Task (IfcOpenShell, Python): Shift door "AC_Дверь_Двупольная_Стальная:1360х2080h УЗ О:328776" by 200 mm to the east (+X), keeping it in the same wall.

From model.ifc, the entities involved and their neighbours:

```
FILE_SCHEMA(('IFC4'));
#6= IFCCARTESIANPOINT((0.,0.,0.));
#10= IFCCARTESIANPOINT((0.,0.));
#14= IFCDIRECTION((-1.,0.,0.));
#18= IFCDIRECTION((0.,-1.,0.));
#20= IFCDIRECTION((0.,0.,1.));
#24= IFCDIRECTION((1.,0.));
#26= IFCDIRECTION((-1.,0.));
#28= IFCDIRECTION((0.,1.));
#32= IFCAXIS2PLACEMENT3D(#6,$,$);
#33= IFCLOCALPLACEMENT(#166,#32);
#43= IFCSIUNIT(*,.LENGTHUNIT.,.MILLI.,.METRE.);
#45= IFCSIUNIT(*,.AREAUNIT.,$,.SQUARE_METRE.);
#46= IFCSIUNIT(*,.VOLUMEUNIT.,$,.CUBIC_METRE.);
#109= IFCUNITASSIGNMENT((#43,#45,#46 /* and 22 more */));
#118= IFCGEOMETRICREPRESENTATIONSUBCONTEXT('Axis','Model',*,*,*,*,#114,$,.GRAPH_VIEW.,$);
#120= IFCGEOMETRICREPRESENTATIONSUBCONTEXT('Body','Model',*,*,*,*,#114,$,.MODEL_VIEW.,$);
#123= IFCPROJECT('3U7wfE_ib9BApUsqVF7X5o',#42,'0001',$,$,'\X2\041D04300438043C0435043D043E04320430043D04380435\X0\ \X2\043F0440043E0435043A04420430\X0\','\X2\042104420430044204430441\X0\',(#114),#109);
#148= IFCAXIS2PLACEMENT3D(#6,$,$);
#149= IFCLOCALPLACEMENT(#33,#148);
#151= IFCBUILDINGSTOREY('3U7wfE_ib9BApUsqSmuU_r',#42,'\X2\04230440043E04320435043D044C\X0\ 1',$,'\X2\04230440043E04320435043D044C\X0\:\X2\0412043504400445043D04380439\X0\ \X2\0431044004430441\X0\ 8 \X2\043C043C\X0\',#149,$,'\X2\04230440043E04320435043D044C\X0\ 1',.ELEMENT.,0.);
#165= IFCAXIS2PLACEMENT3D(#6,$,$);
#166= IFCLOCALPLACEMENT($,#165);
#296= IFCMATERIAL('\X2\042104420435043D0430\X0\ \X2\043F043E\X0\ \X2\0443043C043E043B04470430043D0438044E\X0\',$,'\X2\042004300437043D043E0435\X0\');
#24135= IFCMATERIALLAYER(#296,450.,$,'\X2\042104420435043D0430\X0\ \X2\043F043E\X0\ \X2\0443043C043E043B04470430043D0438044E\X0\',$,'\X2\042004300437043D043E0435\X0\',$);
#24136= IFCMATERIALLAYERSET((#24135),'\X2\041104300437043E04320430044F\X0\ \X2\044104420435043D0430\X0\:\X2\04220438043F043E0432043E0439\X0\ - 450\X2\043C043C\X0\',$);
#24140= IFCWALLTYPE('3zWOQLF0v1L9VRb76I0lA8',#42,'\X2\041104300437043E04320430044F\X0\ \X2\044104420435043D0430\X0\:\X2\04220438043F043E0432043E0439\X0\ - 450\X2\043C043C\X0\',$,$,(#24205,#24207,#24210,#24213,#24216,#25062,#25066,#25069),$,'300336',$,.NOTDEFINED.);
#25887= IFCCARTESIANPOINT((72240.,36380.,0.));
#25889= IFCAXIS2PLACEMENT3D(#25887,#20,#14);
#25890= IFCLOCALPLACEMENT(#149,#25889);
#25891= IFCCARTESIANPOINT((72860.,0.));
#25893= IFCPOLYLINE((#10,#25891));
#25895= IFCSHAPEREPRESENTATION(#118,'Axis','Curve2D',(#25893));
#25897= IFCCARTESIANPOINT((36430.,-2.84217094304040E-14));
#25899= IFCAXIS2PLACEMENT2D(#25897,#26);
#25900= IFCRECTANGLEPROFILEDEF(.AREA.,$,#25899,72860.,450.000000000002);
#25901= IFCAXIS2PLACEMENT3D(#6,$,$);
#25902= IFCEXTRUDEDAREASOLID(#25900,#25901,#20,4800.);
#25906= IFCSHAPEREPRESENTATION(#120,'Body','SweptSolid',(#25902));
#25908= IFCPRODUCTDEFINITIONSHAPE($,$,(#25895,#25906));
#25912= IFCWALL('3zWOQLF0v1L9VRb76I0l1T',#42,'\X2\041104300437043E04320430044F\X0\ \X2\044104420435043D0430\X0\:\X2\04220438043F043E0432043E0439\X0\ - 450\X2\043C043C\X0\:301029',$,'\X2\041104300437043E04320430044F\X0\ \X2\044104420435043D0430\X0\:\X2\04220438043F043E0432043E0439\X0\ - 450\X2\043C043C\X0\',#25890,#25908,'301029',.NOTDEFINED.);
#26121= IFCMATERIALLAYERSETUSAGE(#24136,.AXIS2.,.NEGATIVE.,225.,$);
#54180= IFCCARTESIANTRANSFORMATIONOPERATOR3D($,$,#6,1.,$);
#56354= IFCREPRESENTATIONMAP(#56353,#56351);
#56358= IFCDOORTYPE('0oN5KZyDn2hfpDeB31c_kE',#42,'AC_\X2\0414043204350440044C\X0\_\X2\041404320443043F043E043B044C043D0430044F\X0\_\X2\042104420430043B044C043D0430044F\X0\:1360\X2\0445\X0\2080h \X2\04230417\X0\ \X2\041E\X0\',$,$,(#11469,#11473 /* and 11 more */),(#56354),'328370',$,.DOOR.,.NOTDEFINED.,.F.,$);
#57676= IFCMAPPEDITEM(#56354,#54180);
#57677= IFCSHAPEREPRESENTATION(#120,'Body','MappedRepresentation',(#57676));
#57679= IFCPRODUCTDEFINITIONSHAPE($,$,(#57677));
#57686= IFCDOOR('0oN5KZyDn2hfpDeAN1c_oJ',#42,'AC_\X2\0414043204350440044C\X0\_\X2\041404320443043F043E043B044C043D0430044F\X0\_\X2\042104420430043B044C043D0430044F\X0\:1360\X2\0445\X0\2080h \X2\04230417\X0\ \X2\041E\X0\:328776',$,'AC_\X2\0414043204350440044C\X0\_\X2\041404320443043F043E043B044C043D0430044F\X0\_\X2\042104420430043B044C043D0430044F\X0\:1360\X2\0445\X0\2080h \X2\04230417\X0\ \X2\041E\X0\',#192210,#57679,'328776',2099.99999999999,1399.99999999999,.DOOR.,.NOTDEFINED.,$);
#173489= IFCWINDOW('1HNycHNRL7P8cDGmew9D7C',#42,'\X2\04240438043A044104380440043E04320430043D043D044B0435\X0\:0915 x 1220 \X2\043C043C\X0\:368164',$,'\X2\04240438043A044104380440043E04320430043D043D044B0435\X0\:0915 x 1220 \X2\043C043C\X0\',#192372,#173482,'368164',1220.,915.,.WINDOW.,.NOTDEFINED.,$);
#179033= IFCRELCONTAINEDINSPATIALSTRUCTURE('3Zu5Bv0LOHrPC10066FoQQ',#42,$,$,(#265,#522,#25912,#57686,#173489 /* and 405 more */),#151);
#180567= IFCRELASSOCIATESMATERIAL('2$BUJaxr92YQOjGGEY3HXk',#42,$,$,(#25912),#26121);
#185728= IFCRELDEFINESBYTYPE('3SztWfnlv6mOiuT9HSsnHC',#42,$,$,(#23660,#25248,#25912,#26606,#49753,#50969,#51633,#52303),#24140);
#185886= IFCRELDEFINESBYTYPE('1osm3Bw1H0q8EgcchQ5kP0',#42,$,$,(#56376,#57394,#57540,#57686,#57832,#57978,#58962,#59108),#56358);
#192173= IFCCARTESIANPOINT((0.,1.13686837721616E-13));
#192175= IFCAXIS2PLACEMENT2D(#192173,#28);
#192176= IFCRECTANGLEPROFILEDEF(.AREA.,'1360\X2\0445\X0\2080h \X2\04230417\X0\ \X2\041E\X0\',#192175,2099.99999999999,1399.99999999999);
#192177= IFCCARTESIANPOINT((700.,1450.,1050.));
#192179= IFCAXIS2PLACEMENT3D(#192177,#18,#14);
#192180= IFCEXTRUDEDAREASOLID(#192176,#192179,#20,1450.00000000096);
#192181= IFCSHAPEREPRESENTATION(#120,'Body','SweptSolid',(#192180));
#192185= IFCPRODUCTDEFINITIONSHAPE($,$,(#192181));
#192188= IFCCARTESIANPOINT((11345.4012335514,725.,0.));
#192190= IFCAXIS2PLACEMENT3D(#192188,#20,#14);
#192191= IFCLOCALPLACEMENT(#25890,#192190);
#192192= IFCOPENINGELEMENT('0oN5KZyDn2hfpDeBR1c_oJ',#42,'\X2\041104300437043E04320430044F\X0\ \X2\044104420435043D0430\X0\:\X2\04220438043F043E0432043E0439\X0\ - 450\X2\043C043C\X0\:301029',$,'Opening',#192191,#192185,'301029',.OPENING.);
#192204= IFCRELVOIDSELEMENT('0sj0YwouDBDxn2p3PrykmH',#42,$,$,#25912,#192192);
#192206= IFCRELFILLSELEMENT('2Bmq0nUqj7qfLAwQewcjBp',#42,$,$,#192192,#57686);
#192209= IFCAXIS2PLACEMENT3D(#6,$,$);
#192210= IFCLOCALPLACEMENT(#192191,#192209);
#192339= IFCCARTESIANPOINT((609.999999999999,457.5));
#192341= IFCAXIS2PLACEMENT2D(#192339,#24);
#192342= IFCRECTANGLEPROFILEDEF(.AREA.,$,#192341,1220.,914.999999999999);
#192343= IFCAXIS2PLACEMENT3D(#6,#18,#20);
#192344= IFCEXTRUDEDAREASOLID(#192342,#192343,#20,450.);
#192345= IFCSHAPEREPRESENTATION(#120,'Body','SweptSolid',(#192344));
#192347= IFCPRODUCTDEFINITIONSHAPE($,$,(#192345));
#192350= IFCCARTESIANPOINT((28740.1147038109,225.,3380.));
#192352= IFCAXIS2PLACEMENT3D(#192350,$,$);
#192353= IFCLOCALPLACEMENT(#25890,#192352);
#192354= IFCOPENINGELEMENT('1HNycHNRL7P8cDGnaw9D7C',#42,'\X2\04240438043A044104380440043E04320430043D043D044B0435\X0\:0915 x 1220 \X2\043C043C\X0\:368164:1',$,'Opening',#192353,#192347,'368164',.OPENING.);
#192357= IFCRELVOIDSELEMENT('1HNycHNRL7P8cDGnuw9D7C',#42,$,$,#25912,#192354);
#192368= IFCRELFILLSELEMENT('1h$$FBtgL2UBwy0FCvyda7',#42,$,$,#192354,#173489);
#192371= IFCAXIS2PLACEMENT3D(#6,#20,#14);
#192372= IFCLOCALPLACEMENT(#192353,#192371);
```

```python
import ifcopenshell
import ifcopenshell.api.geometry
import ifcopenshell.util.placement

model = ifcopenshell.open("model.ifc")

door = model.by_guid("0oN5KZyDn2hfpDeAN1c_oJ")
opening = door.FillsVoids[0].RelatingOpeningElement
wall = opening.VoidsElements[0].RelatingBuildingElement

wall_matrix = ifcopenshell.util.placement.get_local_placement(wall.ObjectPlacement)
shift = wall_matrix[:3, 0] * -200.0
before = ifcopenshell.util.placement.get_local_placement(door.ObjectPlacement)[:3, 3].copy()

# The door is placed relative to its opening, so it follows when the opening moves.
matrix = ifcopenshell.util.placement.get_local_placement(opening.ObjectPlacement)
matrix[:3, 3] += shift
ifcopenshell.api.geometry.edit_object_placement(
    model, product=opening, matrix=matrix, is_si=False, should_transform_children=True
)

after = ifcopenshell.util.placement.get_local_placement(door.ObjectPlacement)[:3, 3]
print("door moved by", (after - before).round(3) + 0.0)

model.write("model_rev.ifc")
```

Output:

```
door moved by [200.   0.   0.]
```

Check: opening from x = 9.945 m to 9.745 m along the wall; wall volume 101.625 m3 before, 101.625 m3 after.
